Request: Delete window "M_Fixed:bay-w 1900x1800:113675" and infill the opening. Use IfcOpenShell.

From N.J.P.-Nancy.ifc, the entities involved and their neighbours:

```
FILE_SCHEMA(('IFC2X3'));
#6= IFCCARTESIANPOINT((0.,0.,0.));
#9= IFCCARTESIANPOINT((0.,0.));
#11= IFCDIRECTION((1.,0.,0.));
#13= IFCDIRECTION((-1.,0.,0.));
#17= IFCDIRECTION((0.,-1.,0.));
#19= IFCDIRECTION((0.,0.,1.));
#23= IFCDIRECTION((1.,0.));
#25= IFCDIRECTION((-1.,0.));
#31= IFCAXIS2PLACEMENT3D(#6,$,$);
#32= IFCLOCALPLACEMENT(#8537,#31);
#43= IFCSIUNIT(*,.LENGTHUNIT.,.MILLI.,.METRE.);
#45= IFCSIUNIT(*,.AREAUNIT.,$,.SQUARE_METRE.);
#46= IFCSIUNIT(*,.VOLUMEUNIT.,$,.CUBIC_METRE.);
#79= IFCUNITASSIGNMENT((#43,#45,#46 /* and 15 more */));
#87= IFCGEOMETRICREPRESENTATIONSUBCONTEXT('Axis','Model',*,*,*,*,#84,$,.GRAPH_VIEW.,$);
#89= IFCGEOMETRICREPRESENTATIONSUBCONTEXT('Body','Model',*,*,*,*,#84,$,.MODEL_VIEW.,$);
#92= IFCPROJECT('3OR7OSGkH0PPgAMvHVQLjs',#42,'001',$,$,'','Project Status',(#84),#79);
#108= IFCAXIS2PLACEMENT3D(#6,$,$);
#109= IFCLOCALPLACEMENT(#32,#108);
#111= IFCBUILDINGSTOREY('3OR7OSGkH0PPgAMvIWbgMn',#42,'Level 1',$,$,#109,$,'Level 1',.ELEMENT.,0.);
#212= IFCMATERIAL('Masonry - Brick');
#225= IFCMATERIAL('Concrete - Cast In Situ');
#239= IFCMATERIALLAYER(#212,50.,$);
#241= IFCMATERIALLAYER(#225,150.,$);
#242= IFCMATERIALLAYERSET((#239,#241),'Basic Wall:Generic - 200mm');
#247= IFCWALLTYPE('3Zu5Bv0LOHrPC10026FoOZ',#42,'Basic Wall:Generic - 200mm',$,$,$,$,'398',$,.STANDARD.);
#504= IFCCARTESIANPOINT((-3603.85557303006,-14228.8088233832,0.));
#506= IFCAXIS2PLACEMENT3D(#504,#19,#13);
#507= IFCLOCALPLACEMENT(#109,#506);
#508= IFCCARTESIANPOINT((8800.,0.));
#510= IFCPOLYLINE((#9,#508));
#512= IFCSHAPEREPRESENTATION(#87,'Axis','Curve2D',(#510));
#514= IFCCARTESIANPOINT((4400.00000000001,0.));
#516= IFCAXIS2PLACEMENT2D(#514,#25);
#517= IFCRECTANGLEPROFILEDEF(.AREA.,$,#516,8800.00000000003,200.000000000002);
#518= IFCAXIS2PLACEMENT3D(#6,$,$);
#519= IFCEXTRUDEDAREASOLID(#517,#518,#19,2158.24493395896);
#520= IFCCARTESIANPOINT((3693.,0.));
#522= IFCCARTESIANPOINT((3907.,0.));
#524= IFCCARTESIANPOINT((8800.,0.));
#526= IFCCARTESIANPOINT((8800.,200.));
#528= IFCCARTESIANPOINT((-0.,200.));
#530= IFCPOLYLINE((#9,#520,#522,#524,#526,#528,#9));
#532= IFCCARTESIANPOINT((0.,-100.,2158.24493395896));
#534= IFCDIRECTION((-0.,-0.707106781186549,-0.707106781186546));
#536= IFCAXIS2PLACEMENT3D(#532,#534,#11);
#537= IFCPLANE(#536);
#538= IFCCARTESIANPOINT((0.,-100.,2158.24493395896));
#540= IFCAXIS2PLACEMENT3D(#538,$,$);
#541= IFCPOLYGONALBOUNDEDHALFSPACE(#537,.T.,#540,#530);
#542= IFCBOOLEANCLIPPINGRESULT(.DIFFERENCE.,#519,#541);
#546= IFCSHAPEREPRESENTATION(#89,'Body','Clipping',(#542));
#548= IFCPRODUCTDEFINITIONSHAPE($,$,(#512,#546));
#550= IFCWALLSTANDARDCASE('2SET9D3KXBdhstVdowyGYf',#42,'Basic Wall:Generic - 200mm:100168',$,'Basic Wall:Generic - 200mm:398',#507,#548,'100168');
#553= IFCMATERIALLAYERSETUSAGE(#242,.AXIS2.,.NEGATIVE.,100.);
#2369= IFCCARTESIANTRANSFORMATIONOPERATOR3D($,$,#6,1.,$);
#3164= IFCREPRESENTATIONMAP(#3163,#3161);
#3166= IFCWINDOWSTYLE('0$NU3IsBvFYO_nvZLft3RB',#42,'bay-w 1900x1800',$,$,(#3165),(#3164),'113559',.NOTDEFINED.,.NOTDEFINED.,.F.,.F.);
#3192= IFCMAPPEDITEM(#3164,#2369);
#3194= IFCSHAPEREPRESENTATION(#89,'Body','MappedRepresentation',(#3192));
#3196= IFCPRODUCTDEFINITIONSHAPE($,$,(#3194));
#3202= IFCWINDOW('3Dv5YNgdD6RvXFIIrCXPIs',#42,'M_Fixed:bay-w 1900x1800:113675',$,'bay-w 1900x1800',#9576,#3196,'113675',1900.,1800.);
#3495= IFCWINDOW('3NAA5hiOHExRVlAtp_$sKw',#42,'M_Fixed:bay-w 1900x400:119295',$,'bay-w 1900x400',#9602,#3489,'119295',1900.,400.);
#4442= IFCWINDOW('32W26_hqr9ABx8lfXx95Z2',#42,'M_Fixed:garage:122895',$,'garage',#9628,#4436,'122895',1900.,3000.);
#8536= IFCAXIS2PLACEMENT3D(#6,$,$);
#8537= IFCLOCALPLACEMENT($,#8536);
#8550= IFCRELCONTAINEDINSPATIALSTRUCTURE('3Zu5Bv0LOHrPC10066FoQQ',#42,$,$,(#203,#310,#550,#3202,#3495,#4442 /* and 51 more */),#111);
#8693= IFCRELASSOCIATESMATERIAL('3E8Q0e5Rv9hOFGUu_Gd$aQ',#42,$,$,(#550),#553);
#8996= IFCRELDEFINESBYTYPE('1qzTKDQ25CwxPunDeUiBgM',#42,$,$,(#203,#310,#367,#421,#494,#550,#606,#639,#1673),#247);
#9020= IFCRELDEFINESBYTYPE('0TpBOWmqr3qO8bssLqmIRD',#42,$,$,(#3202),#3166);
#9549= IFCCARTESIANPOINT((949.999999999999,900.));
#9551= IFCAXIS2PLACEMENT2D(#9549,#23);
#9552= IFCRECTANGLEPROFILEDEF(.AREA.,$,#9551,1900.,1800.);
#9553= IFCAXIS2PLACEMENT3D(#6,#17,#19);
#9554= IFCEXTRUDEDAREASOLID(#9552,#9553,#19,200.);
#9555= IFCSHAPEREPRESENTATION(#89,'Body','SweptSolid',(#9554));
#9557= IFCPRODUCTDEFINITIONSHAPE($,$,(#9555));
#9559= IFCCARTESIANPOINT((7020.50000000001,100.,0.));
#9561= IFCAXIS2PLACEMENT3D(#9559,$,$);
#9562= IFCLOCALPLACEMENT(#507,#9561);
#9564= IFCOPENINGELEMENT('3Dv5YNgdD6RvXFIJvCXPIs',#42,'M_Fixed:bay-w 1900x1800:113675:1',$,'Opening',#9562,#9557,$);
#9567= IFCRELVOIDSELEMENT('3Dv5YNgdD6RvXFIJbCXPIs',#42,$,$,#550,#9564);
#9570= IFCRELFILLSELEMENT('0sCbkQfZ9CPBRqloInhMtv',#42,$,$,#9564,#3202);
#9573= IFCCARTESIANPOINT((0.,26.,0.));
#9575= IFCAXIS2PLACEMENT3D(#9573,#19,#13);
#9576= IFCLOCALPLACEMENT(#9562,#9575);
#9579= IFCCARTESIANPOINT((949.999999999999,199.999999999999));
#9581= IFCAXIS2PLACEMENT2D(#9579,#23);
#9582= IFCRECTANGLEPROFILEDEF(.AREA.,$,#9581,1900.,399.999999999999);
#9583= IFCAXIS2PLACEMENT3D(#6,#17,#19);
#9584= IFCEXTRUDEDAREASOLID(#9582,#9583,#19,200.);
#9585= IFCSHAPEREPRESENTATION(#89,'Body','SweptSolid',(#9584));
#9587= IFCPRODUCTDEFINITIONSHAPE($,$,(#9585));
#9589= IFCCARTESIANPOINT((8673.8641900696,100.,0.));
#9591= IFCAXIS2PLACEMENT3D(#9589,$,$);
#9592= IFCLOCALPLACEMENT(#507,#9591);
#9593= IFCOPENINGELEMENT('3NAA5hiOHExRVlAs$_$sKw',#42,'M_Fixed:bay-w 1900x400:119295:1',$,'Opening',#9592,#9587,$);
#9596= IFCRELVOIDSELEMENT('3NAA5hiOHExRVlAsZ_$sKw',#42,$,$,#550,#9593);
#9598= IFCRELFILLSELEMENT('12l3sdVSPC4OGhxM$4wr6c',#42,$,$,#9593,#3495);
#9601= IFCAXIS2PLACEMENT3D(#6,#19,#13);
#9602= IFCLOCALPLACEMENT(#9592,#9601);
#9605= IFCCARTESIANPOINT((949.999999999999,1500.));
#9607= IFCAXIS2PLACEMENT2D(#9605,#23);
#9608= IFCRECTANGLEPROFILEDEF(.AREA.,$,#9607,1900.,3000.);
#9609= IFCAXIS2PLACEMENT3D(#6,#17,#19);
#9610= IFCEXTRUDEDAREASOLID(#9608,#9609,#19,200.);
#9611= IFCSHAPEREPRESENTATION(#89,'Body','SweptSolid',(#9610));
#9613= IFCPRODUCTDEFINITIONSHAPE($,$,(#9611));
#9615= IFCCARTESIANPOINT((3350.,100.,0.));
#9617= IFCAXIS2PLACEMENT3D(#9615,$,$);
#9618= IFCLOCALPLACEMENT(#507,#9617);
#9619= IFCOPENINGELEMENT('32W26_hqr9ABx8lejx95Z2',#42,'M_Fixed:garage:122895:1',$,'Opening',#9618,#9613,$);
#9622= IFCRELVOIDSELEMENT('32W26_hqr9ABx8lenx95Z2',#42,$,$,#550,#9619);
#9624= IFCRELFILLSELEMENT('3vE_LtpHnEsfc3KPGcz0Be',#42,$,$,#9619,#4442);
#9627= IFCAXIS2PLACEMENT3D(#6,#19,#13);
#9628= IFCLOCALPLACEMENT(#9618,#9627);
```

```python
import ifcopenshell
import ifcopenshell.api.feature
import ifcopenshell.api.root
import ifcopenshell.geom
import ifcopenshell.util.shape

model = ifcopenshell.open("N.J.P.-Nancy.ifc")
settings = ifcopenshell.geom.settings()


def volume(element):
    """Net volume in cubic metres, openings subtracted."""
    shape = ifcopenshell.geom.create_shape(settings, element)
    return ifcopenshell.util.shape.get_volume(shape.geometry)


window = model.by_guid("3Dv5YNgdD6RvXFIIrCXPIs")
opening = window.FillsVoids[0].RelatingOpeningElement
wall = opening.VoidsElements[0].RelatingBuildingElement
before = volume(wall)

ifcopenshell.api.root.remove_product(model, product=window)
ifcopenshell.api.feature.remove_feature(model, feature=opening)

after = volume(wall)

print(f"wall volume {before:.3f} -> {after:.3f} m3")

model.write("N.J.P.-Nancy_edited.ifc")
```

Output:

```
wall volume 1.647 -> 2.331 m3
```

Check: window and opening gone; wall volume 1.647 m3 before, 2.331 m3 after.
